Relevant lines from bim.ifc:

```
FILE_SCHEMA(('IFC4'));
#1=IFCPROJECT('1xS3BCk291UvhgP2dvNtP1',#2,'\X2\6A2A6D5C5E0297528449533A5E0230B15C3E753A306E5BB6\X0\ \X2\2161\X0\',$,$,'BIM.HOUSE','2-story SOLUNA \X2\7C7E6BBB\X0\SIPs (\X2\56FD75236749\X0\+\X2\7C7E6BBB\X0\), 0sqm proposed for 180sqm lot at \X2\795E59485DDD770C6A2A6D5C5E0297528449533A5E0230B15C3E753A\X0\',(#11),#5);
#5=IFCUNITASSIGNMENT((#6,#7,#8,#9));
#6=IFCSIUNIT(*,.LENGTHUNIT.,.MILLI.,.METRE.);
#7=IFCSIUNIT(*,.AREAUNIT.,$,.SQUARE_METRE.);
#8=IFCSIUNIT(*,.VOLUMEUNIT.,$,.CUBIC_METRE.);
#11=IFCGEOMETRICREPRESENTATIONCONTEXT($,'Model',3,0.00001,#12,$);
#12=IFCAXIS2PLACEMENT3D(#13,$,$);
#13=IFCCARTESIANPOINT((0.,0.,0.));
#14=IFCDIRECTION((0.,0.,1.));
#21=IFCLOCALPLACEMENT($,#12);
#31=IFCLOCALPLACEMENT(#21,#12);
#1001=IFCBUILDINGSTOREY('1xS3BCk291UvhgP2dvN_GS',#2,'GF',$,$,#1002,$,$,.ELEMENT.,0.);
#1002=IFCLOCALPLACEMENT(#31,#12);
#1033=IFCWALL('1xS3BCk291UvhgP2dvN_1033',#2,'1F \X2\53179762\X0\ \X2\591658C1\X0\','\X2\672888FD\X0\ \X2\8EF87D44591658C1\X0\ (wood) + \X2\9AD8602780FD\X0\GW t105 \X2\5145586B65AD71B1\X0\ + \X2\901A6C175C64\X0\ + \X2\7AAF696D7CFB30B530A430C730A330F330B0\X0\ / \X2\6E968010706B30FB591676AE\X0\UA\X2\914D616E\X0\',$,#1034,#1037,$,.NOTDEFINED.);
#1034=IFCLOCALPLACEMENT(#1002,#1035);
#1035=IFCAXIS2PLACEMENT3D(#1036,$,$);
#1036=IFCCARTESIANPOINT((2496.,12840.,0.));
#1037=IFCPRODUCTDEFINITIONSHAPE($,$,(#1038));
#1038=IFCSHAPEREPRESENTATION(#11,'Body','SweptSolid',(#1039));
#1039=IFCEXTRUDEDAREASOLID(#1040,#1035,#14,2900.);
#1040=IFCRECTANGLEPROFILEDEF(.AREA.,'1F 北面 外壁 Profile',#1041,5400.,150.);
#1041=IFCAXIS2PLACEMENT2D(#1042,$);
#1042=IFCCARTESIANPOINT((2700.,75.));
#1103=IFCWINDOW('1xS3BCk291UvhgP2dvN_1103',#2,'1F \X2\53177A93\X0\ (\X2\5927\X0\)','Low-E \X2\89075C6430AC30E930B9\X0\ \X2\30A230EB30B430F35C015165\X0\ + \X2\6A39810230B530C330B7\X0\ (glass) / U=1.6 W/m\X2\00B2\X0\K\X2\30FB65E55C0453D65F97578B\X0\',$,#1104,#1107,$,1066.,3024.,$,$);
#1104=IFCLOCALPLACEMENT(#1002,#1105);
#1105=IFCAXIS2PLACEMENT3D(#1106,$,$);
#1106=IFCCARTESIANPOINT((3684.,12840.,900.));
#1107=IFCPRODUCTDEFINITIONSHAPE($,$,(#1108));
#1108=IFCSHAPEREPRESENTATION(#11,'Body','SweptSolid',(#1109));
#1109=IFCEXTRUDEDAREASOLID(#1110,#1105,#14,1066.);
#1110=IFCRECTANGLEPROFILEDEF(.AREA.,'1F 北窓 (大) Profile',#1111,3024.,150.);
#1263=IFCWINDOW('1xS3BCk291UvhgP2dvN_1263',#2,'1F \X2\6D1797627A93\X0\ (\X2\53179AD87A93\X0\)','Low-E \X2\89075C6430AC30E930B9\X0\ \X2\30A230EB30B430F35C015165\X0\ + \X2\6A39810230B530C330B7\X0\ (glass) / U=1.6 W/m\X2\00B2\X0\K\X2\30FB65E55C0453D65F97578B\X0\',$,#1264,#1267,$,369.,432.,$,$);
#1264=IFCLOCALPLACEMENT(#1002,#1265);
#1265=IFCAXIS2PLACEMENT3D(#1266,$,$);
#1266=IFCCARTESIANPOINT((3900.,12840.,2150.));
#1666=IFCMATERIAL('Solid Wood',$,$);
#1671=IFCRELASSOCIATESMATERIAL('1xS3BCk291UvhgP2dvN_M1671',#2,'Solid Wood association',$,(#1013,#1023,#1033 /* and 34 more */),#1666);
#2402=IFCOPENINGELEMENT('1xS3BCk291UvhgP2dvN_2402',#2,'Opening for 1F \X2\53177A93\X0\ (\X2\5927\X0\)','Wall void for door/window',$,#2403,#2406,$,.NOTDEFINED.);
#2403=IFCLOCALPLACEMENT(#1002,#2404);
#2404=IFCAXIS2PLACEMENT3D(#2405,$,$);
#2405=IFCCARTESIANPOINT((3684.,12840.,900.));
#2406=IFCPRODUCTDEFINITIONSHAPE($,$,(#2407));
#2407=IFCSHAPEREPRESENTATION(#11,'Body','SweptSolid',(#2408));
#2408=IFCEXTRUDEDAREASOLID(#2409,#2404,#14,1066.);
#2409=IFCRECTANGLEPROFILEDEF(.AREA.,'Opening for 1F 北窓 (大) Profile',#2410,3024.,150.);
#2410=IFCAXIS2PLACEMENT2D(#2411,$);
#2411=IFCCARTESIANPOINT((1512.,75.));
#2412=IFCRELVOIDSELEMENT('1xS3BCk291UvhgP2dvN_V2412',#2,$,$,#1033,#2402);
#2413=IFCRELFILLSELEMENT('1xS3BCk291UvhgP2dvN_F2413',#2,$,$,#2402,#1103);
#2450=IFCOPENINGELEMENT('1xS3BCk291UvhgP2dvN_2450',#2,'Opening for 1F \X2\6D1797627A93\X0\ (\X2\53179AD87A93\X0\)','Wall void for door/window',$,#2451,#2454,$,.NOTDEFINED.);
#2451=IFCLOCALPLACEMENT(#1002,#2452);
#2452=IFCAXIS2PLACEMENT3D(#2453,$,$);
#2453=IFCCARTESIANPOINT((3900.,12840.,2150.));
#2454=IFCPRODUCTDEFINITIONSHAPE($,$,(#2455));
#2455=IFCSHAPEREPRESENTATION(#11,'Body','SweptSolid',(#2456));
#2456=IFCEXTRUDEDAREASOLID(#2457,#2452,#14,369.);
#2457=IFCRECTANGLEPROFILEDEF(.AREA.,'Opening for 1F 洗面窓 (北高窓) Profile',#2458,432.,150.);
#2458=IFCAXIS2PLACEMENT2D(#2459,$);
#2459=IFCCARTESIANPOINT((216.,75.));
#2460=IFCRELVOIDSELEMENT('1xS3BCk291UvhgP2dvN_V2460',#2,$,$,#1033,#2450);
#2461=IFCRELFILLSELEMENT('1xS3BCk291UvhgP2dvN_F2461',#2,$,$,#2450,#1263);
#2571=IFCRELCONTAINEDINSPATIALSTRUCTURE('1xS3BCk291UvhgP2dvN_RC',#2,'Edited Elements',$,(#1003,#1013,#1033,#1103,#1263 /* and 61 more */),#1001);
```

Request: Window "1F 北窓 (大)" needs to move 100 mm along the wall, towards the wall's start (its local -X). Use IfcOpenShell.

```python
import ifcopenshell
import ifcopenshell.api.geometry
import ifcopenshell.util.placement

model = ifcopenshell.open("bim.ifc")

window = model.by_guid("1xS3BCk291UvhgP2dvN_1103")
opening = window.FillsVoids[0].RelatingOpeningElement
wall = opening.VoidsElements[0].RelatingBuildingElement

wall_matrix = ifcopenshell.util.placement.get_local_placement(wall.ObjectPlacement)
shift = wall_matrix[:3, 0] * -100.0
before = ifcopenshell.util.placement.get_local_placement(window.ObjectPlacement)[:3, 3].copy()

# The window is not placed relative to its opening, so move both.
for product in (opening, window):
    matrix = ifcopenshell.util.placement.get_local_placement(product.ObjectPlacement)
    matrix[:3, 3] += shift
    ifcopenshell.api.geometry.edit_object_placement(model, product=product, matrix=matrix, is_si=False)

after = ifcopenshell.util.placement.get_local_placement(window.ObjectPlacement)[:3, 3]
print("window moved by", (after - before).round(3) + 0.0)

model.write("bim_updated.ifc")
```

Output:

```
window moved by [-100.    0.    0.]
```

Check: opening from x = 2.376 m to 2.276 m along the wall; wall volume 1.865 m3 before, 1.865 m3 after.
